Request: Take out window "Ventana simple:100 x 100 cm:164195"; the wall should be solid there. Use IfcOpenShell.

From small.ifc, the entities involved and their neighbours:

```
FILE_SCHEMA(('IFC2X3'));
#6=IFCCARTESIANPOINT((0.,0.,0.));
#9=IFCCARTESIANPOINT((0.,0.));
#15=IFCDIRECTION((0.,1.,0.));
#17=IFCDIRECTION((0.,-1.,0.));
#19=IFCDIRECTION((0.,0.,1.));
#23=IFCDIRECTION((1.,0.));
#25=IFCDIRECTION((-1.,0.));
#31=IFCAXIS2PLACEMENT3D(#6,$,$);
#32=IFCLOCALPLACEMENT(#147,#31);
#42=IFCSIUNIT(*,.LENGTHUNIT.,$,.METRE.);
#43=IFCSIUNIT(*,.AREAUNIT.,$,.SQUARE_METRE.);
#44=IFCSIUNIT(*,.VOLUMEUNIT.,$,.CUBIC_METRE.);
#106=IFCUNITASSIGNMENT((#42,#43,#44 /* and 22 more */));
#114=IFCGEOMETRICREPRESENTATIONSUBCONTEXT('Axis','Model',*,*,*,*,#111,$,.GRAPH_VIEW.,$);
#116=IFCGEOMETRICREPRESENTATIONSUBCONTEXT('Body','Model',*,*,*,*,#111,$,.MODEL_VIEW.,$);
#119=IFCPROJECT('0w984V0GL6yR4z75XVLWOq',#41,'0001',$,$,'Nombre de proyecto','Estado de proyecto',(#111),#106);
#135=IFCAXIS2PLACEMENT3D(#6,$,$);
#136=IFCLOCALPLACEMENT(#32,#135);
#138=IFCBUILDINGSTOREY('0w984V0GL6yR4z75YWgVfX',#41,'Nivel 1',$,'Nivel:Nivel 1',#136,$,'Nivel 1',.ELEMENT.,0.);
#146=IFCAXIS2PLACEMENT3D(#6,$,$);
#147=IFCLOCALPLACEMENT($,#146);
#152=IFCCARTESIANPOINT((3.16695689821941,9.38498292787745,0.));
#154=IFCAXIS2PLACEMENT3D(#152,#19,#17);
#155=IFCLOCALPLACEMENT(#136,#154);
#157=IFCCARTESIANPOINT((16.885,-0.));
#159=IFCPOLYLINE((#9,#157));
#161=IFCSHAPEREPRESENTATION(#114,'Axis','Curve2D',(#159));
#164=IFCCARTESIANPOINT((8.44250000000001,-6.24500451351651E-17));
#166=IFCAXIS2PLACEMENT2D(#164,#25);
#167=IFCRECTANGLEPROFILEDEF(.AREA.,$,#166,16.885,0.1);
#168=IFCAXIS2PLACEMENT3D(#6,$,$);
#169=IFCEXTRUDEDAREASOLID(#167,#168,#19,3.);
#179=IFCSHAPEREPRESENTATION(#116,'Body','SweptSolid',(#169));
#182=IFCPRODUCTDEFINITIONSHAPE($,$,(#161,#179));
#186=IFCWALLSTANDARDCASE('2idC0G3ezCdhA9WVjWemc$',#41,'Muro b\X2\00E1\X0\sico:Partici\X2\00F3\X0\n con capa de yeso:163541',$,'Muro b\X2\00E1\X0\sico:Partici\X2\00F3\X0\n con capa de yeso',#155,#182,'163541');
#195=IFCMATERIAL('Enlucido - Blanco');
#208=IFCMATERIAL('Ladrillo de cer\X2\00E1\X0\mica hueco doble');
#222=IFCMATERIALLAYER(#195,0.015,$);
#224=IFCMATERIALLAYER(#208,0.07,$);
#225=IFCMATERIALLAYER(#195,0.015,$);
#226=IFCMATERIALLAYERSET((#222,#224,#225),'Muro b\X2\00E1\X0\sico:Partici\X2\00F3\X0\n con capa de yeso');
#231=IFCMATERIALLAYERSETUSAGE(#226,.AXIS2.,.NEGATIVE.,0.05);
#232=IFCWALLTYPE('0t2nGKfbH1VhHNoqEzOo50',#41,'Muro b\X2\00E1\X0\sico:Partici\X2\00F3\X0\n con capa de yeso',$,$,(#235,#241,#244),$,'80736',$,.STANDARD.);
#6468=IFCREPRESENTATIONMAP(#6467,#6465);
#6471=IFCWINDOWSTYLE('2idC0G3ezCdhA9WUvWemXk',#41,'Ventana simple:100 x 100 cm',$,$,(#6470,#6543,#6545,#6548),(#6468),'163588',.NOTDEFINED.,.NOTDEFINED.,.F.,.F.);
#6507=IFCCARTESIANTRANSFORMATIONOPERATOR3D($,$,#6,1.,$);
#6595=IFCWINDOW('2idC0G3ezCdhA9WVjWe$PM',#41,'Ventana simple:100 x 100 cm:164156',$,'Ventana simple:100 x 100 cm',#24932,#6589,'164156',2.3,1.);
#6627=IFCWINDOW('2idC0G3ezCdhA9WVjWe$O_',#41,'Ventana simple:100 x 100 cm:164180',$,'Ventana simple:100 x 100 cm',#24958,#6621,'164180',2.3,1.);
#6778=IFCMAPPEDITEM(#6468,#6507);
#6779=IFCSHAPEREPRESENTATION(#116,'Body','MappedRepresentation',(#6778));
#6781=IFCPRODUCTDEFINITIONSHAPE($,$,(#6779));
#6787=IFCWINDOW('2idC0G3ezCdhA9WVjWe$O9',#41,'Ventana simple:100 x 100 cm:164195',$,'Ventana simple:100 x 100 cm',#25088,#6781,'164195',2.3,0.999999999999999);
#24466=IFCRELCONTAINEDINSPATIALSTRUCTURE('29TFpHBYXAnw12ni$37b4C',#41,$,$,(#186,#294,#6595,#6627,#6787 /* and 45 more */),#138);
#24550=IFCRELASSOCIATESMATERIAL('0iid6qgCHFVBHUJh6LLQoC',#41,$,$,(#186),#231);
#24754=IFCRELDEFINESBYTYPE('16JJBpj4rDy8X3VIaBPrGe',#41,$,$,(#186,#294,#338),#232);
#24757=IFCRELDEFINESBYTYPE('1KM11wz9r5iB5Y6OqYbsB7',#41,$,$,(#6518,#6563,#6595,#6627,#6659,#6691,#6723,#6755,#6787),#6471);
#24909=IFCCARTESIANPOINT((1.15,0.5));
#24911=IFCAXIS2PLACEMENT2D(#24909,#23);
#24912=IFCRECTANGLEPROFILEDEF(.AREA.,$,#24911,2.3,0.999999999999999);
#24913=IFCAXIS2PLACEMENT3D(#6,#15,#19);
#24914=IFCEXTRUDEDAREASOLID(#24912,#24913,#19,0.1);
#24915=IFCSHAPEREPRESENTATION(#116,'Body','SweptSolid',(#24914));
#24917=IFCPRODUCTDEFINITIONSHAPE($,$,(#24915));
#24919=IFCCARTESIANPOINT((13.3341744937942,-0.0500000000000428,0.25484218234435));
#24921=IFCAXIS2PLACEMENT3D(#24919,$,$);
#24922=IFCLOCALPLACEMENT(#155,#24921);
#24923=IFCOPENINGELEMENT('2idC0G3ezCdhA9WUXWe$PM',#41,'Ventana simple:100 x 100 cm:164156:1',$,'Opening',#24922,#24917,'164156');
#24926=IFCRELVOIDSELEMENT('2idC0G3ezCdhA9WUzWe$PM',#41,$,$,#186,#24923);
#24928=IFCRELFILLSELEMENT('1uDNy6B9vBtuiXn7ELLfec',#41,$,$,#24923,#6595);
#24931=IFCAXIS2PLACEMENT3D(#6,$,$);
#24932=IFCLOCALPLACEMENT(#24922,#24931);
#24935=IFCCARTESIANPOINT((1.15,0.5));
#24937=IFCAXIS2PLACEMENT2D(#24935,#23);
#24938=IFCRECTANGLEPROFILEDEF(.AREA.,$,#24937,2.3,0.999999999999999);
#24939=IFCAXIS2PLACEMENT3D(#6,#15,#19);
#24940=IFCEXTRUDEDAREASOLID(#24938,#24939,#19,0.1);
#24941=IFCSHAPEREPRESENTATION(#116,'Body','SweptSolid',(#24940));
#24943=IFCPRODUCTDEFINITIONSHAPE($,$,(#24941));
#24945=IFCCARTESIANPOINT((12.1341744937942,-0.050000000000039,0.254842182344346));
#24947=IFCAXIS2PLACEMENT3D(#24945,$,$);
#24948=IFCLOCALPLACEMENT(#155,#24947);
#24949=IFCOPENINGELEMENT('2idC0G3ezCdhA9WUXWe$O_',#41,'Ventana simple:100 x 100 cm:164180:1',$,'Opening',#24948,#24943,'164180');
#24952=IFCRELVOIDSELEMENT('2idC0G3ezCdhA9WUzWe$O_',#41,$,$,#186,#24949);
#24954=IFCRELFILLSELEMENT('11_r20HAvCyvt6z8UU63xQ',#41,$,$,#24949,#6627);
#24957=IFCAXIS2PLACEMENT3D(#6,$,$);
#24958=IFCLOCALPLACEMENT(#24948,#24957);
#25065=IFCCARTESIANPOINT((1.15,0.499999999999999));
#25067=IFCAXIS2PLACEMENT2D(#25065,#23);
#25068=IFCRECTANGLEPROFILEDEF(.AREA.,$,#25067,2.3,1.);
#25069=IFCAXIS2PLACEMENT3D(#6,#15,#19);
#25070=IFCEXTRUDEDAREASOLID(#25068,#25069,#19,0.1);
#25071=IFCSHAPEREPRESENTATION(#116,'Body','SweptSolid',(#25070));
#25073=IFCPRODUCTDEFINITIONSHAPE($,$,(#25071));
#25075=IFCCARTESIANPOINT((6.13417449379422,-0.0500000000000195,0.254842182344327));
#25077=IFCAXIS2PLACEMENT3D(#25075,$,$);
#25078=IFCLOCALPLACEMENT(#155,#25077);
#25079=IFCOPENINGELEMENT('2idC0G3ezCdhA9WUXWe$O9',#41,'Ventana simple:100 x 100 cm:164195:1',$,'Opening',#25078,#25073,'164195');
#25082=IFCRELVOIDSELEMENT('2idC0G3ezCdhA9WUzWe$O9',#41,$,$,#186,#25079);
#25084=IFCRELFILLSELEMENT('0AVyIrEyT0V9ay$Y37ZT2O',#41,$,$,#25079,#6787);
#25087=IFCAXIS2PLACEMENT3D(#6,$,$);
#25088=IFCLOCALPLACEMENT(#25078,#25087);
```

```python
import ifcopenshell
import ifcopenshell.api.feature
import ifcopenshell.api.root
import ifcopenshell.geom
import ifcopenshell.util.shape

model = ifcopenshell.open("small.ifc")
settings = ifcopenshell.geom.settings()


def volume(element):
    """Net volume in cubic metres, openings subtracted."""
    shape = ifcopenshell.geom.create_shape(settings, element)
    return ifcopenshell.util.shape.get_volume(shape.geometry)


window = model.by_guid("2idC0G3ezCdhA9WVjWe$O9")
opening = window.FillsVoids[0].RelatingOpeningElement
wall = opening.VoidsElements[0].RelatingBuildingElement
before = volume(wall)

ifcopenshell.api.root.remove_product(model, product=window)
ifcopenshell.api.feature.remove_feature(model, feature=opening)

after = volume(wall)

print(f"wall volume {before:.3f} -> {after:.3f} m3")

model.write("small_rev.ifc")
```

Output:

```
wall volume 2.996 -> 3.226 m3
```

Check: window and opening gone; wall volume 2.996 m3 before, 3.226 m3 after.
